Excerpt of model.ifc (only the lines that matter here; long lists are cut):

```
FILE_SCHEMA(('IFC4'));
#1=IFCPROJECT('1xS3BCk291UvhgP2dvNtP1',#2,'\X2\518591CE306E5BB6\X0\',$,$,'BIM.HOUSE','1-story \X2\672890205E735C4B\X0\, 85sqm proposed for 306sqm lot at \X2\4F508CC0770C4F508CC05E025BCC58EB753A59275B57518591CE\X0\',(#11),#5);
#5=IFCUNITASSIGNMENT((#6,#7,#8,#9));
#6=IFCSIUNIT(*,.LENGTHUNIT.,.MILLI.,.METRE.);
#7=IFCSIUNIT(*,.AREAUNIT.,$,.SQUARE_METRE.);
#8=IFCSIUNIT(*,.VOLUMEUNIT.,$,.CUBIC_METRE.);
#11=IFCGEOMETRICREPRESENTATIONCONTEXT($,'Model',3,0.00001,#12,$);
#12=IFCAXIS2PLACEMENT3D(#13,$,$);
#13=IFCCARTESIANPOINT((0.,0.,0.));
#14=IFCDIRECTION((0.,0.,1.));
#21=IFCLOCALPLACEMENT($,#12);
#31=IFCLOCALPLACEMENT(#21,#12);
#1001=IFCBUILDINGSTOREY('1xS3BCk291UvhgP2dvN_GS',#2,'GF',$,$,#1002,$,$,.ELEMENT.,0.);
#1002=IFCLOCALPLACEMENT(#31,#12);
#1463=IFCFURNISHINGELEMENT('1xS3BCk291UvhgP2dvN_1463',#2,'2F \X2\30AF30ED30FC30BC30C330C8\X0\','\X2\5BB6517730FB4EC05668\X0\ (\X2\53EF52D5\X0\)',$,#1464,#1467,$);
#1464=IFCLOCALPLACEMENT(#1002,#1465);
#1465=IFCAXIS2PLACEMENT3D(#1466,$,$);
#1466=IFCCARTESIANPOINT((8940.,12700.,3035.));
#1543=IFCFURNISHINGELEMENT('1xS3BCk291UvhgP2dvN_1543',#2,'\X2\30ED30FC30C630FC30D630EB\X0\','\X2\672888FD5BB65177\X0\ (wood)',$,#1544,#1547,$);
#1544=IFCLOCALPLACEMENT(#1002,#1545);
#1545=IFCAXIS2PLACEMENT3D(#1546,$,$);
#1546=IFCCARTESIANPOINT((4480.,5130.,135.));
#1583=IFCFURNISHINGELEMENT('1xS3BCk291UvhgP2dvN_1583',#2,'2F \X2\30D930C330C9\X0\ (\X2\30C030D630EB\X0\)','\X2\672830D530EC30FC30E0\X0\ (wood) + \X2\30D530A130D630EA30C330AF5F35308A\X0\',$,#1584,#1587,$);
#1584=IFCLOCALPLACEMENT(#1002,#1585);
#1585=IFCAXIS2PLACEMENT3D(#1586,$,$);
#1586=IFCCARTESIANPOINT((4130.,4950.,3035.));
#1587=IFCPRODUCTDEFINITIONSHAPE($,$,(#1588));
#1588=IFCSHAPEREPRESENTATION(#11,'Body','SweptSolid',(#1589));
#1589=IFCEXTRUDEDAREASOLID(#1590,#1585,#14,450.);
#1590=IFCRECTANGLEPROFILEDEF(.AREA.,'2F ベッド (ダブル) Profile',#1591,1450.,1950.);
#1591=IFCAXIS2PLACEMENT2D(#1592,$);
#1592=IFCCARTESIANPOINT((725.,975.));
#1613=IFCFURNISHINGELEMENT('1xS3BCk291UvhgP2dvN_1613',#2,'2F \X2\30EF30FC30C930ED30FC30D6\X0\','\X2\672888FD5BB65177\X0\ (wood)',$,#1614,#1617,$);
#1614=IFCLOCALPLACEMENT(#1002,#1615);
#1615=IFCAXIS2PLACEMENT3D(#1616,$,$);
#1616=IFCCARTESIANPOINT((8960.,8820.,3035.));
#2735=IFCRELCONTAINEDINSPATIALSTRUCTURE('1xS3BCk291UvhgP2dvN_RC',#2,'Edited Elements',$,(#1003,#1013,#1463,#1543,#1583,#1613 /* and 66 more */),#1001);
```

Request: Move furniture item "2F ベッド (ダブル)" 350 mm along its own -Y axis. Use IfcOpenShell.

```python
import ifcopenshell
import ifcopenshell.api.geometry
import ifcopenshell.util.placement

model = ifcopenshell.open("model.ifc")

item = model.by_guid("1xS3BCk291UvhgP2dvN_1583")
matrix = ifcopenshell.util.placement.get_local_placement(item.ObjectPlacement)
matrix[:3, 3] -= matrix[:3, 1] * 350.0
ifcopenshell.api.geometry.edit_object_placement(model, product=item, matrix=matrix, is_si=False)

print(ifcopenshell.util.placement.get_local_placement(item.ObjectPlacement).round(3) + 0.0)

model.write("model_edited.ifc")
```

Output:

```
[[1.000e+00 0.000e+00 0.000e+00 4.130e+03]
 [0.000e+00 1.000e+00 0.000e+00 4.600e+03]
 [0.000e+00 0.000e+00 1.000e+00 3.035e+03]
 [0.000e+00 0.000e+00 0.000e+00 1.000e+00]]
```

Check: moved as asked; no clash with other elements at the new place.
